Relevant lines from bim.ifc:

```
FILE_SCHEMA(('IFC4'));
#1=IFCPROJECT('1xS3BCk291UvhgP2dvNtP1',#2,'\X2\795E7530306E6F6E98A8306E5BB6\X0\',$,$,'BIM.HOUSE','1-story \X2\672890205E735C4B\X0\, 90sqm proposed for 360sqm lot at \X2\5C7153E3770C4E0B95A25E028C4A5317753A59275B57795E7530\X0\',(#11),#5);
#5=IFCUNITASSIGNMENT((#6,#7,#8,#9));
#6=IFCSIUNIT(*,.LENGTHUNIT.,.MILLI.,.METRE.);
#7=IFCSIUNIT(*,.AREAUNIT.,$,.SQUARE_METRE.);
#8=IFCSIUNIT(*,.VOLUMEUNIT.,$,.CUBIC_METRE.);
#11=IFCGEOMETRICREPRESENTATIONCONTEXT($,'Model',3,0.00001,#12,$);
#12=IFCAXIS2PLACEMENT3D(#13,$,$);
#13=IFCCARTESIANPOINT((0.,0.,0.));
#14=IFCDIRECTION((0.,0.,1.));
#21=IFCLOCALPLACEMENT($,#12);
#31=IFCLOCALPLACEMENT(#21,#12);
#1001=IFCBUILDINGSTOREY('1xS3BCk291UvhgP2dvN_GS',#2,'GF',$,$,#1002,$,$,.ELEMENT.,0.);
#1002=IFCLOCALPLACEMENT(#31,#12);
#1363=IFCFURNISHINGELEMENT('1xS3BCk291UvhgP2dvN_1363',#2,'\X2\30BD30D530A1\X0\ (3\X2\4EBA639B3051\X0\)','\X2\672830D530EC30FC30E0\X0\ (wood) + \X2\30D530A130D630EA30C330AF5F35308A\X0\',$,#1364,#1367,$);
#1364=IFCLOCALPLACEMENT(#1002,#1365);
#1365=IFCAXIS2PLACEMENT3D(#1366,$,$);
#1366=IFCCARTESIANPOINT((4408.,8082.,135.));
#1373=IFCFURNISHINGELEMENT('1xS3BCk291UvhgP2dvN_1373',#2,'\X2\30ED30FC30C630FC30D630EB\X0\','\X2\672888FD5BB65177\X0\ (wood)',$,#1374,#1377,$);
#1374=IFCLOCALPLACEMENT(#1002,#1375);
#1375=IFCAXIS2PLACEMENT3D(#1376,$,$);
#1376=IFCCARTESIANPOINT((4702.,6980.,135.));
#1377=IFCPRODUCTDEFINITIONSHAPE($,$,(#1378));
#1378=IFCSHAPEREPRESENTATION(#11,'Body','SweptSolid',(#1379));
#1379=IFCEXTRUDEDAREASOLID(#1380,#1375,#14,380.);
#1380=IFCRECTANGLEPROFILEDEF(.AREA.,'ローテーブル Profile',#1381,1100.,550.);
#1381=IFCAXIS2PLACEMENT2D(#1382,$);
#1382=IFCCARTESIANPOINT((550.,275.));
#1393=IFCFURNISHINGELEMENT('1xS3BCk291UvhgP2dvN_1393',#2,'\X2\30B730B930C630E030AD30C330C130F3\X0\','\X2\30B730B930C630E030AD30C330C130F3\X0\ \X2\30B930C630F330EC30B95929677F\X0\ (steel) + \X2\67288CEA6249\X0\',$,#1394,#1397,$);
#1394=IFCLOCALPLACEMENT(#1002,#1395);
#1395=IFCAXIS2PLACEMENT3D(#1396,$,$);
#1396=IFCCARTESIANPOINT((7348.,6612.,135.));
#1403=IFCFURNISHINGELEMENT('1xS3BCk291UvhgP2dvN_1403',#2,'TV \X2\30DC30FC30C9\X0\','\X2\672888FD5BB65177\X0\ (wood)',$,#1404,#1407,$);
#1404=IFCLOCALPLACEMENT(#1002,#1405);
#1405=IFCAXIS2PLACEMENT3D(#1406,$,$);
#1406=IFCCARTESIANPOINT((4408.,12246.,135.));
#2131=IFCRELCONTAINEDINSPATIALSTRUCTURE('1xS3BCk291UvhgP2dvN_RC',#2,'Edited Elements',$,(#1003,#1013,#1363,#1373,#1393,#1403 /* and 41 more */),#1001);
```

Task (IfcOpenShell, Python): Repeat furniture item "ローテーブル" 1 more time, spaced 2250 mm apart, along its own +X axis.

```python
import ifcopenshell
import ifcopenshell.api.geometry
import ifcopenshell.api.root
import ifcopenshell.util.element
import ifcopenshell.util.placement
import ifcopenshell.util.unit

model = ifcopenshell.open("bim.ifc")
unit_scale = ifcopenshell.util.unit.calculate_unit_scale(model)


def reuse_history(source, copy):
    """copy_class also copies each property set's owner history, people and application; keep the originals."""
    for rel in copy.IsDefinedBy:
        if rel.is_a("IfcRelDefinesByProperties") and (history := rel.RelatingPropertyDefinition.OwnerHistory):
            rel.RelatingPropertyDefinition.OwnerHistory = source.OwnerHistory
            ifcopenshell.util.element.remove_deep2(model, history)


source = model.by_guid("1xS3BCk291UvhgP2dvN_1373")
base = ifcopenshell.util.placement.get_local_placement(source.ObjectPlacement)
step = base[:3, 0] * 2.25 / unit_scale

for i in range(1, 2):
    copy = ifcopenshell.api.root.copy_class(model, product=source)
    copy.Representation = ifcopenshell.util.element.copy_deep(
        model, source.Representation, exclude=["IfcGeometricRepresentationContext", "IfcRepresentationMap"]
    )
    reuse_history(source, copy)
    matrix = base.copy()
    matrix[:3, 3] += i * step
    print("added at", matrix[:3, 3].round(3) + 0.0)
    ifcopenshell.api.geometry.edit_object_placement(model, product=copy, matrix=matrix, is_si=False)

model.write("bim_edited.ifc")
```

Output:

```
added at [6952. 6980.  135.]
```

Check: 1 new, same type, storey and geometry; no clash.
